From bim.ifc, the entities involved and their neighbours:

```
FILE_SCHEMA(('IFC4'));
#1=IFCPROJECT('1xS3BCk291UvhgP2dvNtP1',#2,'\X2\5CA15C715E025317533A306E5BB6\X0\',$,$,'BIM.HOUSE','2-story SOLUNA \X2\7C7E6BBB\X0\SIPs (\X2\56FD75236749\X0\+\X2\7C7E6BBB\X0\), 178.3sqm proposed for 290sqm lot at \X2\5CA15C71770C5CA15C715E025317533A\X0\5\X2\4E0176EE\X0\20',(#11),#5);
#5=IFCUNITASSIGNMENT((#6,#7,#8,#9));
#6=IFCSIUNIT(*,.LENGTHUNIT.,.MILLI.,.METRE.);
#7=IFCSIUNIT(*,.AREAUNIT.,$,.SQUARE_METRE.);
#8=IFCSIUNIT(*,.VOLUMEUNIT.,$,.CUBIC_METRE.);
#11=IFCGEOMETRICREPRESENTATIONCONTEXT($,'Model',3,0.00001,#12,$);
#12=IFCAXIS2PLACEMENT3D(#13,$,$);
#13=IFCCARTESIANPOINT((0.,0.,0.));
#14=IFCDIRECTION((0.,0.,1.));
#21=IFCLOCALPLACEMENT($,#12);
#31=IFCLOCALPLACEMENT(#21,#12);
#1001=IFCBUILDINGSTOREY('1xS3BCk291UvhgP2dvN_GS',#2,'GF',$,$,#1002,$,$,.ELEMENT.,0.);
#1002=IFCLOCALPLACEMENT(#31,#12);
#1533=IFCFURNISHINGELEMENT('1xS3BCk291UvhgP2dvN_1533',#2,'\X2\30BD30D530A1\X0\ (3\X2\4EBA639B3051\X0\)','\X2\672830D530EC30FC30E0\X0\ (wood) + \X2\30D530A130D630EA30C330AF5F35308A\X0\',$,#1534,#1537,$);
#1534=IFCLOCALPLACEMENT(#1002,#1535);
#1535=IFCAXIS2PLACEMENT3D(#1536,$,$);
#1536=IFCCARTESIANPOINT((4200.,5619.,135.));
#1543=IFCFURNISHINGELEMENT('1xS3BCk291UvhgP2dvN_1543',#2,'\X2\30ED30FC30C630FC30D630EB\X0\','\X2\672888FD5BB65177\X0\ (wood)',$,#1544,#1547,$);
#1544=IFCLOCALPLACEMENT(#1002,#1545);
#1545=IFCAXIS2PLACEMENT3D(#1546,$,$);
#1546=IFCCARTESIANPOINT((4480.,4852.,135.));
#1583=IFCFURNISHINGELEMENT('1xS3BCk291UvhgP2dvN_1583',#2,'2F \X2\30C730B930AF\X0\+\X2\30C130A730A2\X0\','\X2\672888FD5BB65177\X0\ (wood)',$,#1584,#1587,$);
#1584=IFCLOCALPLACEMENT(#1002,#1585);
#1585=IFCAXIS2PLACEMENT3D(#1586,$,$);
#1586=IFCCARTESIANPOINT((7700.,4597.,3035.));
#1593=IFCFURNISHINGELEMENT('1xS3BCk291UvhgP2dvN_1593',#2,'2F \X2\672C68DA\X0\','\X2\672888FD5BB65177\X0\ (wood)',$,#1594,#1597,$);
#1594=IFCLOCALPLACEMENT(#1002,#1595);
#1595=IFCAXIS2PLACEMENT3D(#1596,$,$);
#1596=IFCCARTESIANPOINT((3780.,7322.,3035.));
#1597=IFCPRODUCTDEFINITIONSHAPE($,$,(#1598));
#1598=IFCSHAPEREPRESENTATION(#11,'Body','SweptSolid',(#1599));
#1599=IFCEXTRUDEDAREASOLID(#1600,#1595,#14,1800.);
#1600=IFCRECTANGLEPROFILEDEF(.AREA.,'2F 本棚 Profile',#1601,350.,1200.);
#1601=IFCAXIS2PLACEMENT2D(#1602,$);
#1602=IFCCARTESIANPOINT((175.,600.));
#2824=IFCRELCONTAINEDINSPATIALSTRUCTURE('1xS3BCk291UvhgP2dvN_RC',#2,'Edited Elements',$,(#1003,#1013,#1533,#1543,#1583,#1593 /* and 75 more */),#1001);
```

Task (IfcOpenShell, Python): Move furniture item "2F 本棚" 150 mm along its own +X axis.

```python
import ifcopenshell
import ifcopenshell.api.geometry
import ifcopenshell.util.placement

model = ifcopenshell.open("bim.ifc")

item = model.by_guid("1xS3BCk291UvhgP2dvN_1593")
matrix = ifcopenshell.util.placement.get_local_placement(item.ObjectPlacement)
matrix[:3, 3] += matrix[:3, 0] * 150.0
ifcopenshell.api.geometry.edit_object_placement(model, product=item, matrix=matrix, is_si=False)

print(ifcopenshell.util.placement.get_local_placement(item.ObjectPlacement).round(3) + 0.0)

model.write("bim_edited.ifc")
```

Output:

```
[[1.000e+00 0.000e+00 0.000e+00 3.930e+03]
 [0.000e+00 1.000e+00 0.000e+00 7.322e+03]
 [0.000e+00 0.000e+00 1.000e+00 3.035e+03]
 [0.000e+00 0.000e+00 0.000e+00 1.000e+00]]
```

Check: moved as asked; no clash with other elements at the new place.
